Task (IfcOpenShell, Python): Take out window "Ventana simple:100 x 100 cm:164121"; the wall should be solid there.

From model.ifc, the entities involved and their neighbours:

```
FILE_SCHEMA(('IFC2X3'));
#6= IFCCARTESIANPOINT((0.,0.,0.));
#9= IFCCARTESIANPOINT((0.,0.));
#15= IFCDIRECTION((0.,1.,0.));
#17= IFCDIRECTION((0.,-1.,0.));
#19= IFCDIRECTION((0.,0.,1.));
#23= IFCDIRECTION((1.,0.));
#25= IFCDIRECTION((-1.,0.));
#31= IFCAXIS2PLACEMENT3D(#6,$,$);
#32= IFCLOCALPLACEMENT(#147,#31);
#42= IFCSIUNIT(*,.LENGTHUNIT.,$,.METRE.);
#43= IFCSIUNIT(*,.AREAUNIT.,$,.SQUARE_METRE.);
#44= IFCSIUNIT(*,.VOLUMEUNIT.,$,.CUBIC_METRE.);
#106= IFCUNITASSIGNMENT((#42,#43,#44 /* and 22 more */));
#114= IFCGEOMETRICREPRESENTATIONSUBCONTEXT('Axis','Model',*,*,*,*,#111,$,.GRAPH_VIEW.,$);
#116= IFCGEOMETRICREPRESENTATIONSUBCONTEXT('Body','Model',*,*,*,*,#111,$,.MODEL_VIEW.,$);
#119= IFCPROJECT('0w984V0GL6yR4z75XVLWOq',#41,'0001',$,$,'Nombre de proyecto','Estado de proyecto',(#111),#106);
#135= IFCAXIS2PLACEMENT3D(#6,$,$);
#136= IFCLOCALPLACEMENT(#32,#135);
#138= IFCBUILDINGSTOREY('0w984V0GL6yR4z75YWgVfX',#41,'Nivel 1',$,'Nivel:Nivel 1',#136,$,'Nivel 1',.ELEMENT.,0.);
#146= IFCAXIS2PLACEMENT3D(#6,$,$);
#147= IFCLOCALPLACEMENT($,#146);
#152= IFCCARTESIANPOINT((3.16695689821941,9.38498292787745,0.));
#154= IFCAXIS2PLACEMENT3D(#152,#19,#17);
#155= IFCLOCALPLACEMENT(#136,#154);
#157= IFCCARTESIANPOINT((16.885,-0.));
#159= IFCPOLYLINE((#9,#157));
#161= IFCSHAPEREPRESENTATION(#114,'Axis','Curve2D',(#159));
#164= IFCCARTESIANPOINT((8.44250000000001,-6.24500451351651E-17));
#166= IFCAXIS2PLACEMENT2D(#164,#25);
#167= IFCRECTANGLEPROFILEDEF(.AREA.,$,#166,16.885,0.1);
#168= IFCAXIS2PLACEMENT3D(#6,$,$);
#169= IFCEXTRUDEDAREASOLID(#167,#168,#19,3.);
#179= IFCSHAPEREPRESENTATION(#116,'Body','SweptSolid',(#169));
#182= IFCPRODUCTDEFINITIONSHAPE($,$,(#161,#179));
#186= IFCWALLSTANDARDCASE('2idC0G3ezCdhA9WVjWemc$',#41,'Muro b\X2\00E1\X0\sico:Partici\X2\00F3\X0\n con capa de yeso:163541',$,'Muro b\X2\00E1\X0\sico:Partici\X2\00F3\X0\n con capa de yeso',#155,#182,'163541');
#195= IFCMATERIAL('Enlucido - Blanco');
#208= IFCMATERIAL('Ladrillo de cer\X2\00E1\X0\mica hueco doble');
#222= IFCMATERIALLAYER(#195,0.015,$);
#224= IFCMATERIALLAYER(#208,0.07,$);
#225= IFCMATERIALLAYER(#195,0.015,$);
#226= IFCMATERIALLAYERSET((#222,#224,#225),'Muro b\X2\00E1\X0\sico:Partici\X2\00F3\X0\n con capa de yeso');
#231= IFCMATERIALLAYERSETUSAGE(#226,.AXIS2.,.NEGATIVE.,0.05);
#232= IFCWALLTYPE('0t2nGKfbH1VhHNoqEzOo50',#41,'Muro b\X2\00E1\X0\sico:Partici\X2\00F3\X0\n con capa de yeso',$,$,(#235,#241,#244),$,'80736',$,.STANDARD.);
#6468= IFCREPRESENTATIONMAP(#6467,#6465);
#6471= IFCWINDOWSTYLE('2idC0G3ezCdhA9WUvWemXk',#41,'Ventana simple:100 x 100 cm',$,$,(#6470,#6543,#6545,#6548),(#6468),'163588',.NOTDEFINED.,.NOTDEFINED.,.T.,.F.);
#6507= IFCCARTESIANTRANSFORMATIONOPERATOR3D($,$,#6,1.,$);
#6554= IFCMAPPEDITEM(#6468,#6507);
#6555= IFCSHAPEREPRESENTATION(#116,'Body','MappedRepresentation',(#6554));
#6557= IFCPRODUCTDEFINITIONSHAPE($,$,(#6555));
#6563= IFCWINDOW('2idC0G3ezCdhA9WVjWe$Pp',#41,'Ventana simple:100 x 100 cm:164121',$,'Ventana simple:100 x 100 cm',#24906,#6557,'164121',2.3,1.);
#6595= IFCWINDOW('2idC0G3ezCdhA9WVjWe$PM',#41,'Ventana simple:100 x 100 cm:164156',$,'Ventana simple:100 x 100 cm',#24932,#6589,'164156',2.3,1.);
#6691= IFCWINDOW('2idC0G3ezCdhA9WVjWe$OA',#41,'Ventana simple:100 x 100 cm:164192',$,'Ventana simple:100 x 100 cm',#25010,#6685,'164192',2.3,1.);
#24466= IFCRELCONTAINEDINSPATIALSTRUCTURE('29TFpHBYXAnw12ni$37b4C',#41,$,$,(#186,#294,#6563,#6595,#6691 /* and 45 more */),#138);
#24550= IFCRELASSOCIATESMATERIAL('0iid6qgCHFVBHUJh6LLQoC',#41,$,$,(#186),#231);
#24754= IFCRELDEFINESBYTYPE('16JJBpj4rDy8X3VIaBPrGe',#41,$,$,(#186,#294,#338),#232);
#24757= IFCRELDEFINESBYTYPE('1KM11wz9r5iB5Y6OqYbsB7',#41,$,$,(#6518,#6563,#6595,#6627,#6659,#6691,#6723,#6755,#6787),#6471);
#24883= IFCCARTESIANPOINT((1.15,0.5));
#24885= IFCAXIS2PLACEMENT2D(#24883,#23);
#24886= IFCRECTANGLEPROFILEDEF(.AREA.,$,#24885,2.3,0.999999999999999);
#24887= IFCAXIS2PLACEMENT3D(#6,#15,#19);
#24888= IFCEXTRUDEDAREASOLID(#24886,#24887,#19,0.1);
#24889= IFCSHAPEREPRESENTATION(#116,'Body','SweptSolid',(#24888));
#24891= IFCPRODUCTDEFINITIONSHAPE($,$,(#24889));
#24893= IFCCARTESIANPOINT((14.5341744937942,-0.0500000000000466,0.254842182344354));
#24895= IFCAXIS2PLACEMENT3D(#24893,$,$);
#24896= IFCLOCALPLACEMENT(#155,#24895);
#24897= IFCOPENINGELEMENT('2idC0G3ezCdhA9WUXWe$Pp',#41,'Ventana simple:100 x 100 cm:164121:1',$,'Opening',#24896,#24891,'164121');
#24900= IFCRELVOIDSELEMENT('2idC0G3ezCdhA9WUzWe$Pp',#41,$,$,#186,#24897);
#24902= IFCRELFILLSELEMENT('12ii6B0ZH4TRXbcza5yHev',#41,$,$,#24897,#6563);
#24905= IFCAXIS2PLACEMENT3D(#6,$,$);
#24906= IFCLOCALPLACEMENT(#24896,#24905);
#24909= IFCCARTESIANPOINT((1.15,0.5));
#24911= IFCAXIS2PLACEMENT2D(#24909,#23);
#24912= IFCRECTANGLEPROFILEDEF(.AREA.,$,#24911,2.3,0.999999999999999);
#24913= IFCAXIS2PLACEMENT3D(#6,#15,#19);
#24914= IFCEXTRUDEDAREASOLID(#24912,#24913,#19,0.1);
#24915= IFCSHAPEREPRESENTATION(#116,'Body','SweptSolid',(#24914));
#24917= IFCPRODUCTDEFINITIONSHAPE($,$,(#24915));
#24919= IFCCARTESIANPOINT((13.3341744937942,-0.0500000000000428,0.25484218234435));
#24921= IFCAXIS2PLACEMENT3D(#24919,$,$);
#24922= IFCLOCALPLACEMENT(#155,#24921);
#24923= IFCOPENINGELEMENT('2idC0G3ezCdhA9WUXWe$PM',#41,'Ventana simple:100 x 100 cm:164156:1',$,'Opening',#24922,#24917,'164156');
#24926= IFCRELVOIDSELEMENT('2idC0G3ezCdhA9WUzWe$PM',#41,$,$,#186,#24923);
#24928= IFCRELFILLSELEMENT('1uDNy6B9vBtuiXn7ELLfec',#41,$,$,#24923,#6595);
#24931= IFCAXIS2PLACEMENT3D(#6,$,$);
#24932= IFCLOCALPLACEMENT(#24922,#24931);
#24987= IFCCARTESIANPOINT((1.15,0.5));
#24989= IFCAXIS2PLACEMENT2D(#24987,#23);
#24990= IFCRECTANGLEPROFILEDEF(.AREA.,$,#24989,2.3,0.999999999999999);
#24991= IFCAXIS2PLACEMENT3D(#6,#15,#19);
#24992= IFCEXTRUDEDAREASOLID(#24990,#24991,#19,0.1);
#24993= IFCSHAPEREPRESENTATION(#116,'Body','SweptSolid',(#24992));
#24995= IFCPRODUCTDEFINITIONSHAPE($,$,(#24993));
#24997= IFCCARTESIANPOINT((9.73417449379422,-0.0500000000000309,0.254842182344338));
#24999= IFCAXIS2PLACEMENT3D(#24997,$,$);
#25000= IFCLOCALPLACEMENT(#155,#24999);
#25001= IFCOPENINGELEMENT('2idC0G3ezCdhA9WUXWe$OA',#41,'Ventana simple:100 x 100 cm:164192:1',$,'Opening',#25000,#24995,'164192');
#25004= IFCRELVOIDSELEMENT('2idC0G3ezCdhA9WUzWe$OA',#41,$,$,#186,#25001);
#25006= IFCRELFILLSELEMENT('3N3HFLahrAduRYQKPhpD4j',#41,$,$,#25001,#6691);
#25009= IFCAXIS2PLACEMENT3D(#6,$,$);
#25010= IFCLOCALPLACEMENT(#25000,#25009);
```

```python
import ifcopenshell
import ifcopenshell.api.feature
import ifcopenshell.api.root
import ifcopenshell.geom
import ifcopenshell.util.shape

model = ifcopenshell.open("model.ifc")
settings = ifcopenshell.geom.settings()


def volume(element):
    """Net volume in cubic metres, openings subtracted."""
    shape = ifcopenshell.geom.create_shape(settings, element)
    return ifcopenshell.util.shape.get_volume(shape.geometry)


window = model.by_guid("2idC0G3ezCdhA9WVjWe$Pp")
opening = window.FillsVoids[0].RelatingOpeningElement
wall = opening.VoidsElements[0].RelatingBuildingElement
before = volume(wall)

ifcopenshell.api.root.remove_product(model, product=window)
ifcopenshell.api.feature.remove_feature(model, feature=opening)

after = volume(wall)

print(f"wall volume {before:.3f} -> {after:.3f} m3")

model.write("model_v2.ifc")
```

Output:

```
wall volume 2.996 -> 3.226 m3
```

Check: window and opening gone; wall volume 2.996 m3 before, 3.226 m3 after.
